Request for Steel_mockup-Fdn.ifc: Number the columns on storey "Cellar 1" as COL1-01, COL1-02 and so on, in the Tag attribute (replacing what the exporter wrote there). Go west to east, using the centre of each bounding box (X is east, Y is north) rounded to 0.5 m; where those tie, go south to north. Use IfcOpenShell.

First a look at what the model holds.

```python
import ifcopenshell
import ifcopenshell.util.element
import ifcopenshell.util.placement

model = ifcopenshell.open("Steel_mockup-Fdn.ifc")
print(model.schema)
storey = next(s for s in model.by_type("IfcBuildingStorey") if s.Name == "Cellar 1")
columns = [e for e in ifcopenshell.util.element.get_decomposition(storey) if e.is_a("IfcColumn")]
for e in sorted(columns, key=lambda e: e.id()):
    origin = ifcopenshell.util.placement.get_local_placement(e.ObjectPlacement)[:3, 3]
    print(e.id(), e.Tag, e.Name, origin.round(2) + 0.0, sep=" | ")
```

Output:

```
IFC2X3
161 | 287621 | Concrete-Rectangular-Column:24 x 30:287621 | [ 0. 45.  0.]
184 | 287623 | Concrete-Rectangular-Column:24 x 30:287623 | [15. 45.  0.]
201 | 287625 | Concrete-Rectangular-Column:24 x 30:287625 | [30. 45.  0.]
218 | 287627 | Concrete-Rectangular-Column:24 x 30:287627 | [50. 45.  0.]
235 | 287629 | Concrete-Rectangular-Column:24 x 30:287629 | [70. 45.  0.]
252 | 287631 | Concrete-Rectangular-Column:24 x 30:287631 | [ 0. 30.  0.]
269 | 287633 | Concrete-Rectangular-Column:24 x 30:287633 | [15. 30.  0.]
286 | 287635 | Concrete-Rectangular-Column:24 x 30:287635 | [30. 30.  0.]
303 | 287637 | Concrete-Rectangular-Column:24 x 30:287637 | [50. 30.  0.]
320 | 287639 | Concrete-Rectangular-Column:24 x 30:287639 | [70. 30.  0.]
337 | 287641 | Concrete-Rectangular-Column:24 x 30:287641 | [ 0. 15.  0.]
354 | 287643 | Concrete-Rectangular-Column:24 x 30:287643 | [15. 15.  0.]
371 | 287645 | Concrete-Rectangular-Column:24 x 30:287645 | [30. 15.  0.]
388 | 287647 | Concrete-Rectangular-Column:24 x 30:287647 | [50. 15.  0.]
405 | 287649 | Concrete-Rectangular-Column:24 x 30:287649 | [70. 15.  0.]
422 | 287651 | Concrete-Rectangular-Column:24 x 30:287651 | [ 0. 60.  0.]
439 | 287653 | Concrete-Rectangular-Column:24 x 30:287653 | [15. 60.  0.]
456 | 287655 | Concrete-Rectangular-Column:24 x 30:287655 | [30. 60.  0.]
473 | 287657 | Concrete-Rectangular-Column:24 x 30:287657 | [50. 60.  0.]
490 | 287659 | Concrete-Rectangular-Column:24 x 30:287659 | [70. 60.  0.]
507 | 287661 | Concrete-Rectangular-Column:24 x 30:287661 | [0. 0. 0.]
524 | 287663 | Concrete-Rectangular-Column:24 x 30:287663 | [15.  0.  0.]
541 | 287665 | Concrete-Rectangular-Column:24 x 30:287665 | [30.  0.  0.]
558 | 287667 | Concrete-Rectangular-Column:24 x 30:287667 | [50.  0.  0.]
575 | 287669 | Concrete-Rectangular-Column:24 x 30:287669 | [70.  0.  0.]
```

```python
import ifcopenshell
import ifcopenshell.geom
import ifcopenshell.util.element
import ifcopenshell.util.shape

model = ifcopenshell.open("Steel_mockup-Fdn.ifc")
settings = ifcopenshell.geom.settings()
settings.set("use-world-coords", True)


def centre(element):
    shape = ifcopenshell.geom.create_shape(settings, element)
    return ifcopenshell.util.shape.get_bbox_centroid(shape.geometry)


storey = next(s for s in model.by_type("IfcBuildingStorey") if s.Name == "Cellar 1")
columns = [e for e in ifcopenshell.util.element.get_decomposition(storey) if e.is_a("IfcColumn")]

# Insertion points can sit at a corner or the storey origin, so sort by the geometry (in metres).
centres = {e: centre(e) for e in columns}
columns.sort(key=lambda e: (round(centres[e][0] / 0.5), centres[e][1]))

for i, e in enumerate(columns, start=1):
    number = f"COL1-{i:02d}"
    e.Tag = number
    print(e.id(), number)

model.write("Steel_mockup-Fdn_updated.ifc")
```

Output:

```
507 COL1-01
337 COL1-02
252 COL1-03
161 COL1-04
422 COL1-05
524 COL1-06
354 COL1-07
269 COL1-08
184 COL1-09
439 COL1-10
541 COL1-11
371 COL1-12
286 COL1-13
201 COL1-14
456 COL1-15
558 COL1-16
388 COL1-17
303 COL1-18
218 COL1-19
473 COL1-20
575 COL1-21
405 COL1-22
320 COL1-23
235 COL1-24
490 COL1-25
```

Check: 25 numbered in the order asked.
